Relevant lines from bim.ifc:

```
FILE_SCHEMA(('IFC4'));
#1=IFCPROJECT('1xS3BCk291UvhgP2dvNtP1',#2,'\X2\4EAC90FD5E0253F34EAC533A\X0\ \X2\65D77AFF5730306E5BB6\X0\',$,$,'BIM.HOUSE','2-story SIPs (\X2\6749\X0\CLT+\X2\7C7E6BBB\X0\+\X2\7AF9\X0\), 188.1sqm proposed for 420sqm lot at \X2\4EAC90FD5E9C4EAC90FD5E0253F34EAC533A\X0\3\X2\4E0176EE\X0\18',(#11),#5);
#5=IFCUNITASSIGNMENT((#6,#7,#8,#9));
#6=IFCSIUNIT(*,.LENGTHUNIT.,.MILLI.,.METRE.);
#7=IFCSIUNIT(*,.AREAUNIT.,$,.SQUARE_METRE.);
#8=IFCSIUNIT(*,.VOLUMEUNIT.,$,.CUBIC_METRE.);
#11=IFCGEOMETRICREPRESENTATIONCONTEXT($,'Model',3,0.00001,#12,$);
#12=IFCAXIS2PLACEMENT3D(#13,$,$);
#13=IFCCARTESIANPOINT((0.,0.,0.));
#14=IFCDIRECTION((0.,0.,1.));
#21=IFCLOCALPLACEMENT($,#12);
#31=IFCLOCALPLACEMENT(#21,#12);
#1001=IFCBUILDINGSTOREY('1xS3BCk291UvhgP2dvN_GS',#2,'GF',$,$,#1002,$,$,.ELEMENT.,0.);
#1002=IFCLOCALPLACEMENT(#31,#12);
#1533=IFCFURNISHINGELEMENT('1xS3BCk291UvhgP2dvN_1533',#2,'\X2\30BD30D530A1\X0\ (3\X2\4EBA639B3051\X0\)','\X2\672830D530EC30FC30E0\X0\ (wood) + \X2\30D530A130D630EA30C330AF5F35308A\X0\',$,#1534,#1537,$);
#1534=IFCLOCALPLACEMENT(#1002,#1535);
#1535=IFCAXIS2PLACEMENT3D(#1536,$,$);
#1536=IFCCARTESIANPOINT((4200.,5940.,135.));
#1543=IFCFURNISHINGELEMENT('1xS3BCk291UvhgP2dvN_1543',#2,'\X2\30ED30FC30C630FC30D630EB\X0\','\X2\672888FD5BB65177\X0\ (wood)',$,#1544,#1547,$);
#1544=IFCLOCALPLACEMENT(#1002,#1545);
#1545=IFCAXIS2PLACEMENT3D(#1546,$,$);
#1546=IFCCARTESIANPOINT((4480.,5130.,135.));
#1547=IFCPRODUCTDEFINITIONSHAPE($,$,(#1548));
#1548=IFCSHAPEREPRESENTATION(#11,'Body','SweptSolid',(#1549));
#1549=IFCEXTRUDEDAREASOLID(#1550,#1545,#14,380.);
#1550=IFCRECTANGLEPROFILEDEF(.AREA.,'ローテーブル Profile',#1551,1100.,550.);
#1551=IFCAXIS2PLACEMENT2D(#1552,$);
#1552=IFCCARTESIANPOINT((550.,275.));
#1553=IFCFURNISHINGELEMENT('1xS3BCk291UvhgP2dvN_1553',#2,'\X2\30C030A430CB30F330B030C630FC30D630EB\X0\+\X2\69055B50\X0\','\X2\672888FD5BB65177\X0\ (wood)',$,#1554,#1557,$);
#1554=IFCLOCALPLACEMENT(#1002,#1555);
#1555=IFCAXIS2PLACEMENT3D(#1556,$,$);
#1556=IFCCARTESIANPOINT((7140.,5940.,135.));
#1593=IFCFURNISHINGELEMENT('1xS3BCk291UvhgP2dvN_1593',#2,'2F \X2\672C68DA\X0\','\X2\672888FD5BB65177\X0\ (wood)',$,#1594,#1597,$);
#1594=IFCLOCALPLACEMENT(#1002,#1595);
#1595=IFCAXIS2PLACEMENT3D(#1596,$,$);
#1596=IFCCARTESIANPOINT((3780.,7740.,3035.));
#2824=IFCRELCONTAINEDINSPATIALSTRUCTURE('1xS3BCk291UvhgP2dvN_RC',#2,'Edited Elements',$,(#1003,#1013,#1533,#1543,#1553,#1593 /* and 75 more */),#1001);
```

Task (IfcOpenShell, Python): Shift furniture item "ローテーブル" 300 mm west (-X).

```python
import ifcopenshell
import ifcopenshell.api.geometry
import ifcopenshell.util.placement

model = ifcopenshell.open("bim.ifc")

item = model.by_guid("1xS3BCk291UvhgP2dvN_1543")
matrix = ifcopenshell.util.placement.get_local_placement(item.ObjectPlacement)
matrix[0, 3] -= 300.0
ifcopenshell.api.geometry.edit_object_placement(model, product=item, matrix=matrix, is_si=False)

print(ifcopenshell.util.placement.get_local_placement(item.ObjectPlacement).round(3) + 0.0)

model.write("bim_updated.ifc")
```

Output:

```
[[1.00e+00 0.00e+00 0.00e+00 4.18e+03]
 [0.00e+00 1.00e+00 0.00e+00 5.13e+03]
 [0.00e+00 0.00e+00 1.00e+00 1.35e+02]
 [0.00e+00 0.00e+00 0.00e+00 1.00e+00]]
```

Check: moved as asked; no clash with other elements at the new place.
